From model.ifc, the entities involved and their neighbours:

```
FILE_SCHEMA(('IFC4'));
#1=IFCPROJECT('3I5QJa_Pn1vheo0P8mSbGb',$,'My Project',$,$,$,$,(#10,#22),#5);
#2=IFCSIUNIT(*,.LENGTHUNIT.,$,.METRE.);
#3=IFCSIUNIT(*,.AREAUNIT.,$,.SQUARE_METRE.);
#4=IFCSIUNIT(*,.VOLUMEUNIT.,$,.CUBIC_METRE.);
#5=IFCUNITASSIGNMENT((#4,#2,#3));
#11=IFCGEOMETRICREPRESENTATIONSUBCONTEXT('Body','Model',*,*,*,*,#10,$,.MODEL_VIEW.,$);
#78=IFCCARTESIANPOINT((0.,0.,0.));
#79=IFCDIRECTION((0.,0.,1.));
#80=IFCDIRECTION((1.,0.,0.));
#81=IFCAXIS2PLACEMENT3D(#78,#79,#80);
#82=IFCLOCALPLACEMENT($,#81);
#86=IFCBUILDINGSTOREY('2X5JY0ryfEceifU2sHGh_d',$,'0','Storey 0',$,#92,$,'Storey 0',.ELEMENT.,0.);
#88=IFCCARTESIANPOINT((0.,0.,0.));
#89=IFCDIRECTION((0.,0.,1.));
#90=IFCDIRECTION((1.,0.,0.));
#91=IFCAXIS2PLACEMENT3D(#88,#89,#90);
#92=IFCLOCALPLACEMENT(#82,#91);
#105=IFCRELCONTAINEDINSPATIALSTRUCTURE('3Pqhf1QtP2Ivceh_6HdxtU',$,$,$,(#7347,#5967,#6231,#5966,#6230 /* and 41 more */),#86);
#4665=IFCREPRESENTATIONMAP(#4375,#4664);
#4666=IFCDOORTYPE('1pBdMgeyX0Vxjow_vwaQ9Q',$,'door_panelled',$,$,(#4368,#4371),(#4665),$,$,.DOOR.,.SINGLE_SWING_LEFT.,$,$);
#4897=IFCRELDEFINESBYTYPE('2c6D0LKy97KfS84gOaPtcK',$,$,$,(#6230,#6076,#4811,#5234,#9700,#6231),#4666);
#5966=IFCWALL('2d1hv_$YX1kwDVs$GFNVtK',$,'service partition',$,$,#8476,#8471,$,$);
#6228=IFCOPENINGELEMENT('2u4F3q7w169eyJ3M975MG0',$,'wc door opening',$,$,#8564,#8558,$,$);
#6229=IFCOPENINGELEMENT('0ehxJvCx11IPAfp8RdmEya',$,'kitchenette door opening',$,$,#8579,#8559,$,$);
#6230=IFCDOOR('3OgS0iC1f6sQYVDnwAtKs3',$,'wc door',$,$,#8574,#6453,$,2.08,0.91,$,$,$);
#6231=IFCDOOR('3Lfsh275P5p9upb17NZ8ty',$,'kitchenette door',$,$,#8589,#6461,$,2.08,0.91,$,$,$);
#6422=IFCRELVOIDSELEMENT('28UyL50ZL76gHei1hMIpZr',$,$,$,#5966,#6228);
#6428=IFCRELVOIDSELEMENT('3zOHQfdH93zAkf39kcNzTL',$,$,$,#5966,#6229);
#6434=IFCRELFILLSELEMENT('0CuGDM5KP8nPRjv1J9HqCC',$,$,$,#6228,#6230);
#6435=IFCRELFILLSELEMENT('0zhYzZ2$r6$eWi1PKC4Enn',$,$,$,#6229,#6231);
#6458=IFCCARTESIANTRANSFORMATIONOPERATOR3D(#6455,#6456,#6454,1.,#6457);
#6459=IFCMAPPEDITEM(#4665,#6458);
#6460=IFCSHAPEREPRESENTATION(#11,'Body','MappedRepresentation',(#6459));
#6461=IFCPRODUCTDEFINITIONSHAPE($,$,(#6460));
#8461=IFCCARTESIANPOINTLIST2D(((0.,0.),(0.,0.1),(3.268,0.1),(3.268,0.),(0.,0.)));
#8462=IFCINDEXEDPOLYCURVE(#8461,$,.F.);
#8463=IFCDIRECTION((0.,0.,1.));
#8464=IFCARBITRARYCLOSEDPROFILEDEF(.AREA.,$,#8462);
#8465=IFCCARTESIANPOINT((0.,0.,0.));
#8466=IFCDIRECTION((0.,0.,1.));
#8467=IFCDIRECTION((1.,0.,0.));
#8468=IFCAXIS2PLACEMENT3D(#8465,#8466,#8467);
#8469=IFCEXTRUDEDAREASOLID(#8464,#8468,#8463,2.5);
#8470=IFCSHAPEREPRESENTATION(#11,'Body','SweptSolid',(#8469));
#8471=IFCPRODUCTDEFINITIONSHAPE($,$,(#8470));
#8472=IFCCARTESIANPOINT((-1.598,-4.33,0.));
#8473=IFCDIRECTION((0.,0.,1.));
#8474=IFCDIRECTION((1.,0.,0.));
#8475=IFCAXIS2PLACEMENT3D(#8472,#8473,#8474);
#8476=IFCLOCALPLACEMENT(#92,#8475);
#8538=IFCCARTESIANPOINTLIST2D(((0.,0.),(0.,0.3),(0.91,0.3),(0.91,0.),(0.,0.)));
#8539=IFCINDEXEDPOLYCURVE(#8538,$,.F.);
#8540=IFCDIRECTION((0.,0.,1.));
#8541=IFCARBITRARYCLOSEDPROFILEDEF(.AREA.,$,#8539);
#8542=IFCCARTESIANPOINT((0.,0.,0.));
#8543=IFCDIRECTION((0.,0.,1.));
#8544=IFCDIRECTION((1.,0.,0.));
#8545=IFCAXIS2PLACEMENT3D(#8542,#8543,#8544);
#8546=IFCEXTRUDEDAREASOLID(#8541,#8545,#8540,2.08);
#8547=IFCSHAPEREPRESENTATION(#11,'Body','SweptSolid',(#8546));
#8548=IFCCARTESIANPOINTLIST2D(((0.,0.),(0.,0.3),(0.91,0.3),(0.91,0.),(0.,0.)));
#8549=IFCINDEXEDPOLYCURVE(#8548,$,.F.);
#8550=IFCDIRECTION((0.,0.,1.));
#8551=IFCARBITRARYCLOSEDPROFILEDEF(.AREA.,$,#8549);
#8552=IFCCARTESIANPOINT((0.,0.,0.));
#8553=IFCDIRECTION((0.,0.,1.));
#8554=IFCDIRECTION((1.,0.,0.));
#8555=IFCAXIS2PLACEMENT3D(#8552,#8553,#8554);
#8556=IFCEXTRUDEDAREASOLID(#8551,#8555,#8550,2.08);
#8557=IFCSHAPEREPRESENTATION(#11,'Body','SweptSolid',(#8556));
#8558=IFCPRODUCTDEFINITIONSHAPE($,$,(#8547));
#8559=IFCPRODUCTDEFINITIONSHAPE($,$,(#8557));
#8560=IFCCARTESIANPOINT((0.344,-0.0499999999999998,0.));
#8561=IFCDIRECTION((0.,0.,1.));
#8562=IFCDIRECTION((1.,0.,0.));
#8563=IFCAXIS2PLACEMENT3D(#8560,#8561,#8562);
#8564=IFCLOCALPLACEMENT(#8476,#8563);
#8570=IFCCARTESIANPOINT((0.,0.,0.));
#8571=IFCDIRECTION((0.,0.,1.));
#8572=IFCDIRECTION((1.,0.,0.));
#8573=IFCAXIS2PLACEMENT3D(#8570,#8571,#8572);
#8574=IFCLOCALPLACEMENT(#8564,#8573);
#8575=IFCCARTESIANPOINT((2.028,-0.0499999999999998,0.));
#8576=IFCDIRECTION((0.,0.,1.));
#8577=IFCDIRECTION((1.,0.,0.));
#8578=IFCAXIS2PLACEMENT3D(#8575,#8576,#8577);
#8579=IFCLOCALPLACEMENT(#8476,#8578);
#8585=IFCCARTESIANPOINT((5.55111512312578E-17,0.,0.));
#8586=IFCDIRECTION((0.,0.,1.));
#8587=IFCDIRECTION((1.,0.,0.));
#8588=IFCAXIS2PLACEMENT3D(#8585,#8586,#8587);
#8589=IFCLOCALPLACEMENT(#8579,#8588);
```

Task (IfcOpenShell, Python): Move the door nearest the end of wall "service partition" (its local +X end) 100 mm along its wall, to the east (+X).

```python
import ifcopenshell
import ifcopenshell.api.geometry
import ifcopenshell.util.placement

model = ifcopenshell.open("model.ifc")

door = model.by_id(6231)
opening = door.FillsVoids[0].RelatingOpeningElement
wall = opening.VoidsElements[0].RelatingBuildingElement

wall_matrix = ifcopenshell.util.placement.get_local_placement(wall.ObjectPlacement)
shift = wall_matrix[:3, 0] * 0.1
before = ifcopenshell.util.placement.get_local_placement(door.ObjectPlacement)[:3, 3].copy()

# The door is placed relative to its opening, so it follows when the opening moves.
matrix = ifcopenshell.util.placement.get_local_placement(opening.ObjectPlacement)
matrix[:3, 3] += shift
ifcopenshell.api.geometry.edit_object_placement(
    model, product=opening, matrix=matrix, is_si=False, should_transform_children=True
)

after = ifcopenshell.util.placement.get_local_placement(door.ObjectPlacement)[:3, 3]
print("door moved by", (after - before).round(3) + 0.0)

model.write("model-out.ifc")
```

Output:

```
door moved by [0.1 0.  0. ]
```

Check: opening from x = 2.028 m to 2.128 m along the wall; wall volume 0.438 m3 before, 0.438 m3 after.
